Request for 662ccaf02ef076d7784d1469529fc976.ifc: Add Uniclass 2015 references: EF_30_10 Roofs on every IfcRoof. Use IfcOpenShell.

First a look at what the model holds.

```python
import ifcopenshell

model = ifcopenshell.open("662ccaf02ef076d7784d1469529fc976.ifc")
print(model.schema)
print("classifications:", [c.Name for c in model.by_type("IfcClassification")])
for ifc_class in ("IfcDoor", "IfcRoof", "IfcStair", "IfcWall", "IfcWindow"):
    print(ifc_class, len(model.by_type(ifc_class)))
```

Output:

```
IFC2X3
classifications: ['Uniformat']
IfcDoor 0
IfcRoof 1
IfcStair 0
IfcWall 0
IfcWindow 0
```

```python
import ifcopenshell
import ifcopenshell.api.classification

model = ifcopenshell.open("662ccaf02ef076d7784d1469529fc976.ifc")

# IFC2X3 requires Source and Edition and has no link from the project to the system.
system = model.create_entity("IfcClassification", Source="NBS", Edition="2015", Name="Uniclass 2015")

codes = {
    "IfcRoof": ("EF_30_10", "Roofs"),
}
for ifc_class, (code, name) in codes.items():
    products = model.by_type(ifc_class)
    ifcopenshell.api.classification.add_reference(
        model, products=products, classification=system, identification=code, name=name
    )
    print(code, len(products))

model.write("662ccaf02ef076d7784d1469529fc976_updated.ifc")
```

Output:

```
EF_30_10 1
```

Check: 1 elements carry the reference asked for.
